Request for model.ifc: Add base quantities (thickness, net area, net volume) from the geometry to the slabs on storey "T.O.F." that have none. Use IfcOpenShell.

First a look at what the model holds.

```python
import ifcopenshell
import ifcopenshell.util.element
import ifcopenshell.util.unit

model = ifcopenshell.open("model.ifc")
print(model.schema)
for unit_type in ("LENGTHUNIT", "AREAUNIT", "VOLUMEUNIT"):
    print(unit_type, ifcopenshell.util.unit.calculate_unit_scale(model, unit_type))
storey = next(s for s in model.by_type("IfcBuildingStorey") if s.Name == "T.O.F.")
slabs = [e for e in ifcopenshell.util.element.get_decomposition(storey) if e.is_a("IfcSlab")]
for e in sorted(slabs, key=lambda e: e.id()):
    print(e.id(), e.is_a(), e.Name, list(ifcopenshell.util.element.get_psets(e, qtos_only=True)), sep=" | ")
```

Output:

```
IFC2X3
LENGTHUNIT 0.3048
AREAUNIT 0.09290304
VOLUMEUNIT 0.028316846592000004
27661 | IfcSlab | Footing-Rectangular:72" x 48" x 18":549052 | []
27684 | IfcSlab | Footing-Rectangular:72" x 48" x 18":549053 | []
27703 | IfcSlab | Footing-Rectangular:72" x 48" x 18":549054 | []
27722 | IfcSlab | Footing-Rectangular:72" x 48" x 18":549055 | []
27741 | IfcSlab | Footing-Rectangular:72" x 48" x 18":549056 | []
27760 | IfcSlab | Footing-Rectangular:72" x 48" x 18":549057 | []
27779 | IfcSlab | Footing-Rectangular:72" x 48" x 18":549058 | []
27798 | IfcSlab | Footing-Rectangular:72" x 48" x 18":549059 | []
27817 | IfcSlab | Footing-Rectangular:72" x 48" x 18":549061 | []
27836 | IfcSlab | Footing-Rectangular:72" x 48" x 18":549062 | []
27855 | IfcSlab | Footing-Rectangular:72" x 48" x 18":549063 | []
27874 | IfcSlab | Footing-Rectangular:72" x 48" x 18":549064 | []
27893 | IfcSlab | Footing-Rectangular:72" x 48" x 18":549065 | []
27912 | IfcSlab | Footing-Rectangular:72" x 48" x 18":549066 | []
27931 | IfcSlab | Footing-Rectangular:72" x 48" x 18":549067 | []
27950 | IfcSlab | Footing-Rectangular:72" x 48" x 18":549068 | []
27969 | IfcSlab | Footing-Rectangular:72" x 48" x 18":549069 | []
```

```python
import ifcopenshell
import ifcopenshell.api.pset
import ifcopenshell.geom
import ifcopenshell.util.element
import ifcopenshell.util.shape
import ifcopenshell.util.unit

model = ifcopenshell.open("model.ifc")
unit_scale = ifcopenshell.util.unit.calculate_unit_scale(model)
area_scale = ifcopenshell.util.unit.calculate_unit_scale(model, "AREAUNIT")
volume_scale = ifcopenshell.util.unit.calculate_unit_scale(model, "VOLUMEUNIT")
settings = ifcopenshell.geom.settings()

storey = next(s for s in model.by_type("IfcBuildingStorey") if s.Name == "T.O.F.")
slabs = [e for e in ifcopenshell.util.element.get_decomposition(storey) if e.is_a("IfcSlab")]

for e in sorted(slabs, key=lambda e: e.id()):
    if ifcopenshell.util.element.get_psets(e, qtos_only=True, should_inherit=False):
        continue
    # Geometry comes back in metres, in the element's own axes.
    shape = ifcopenshell.geom.create_shape(settings, e)
    values = {
        "Width": ifcopenshell.util.shape.get_z(shape.geometry) / unit_scale,
        "NetArea": ifcopenshell.util.shape.get_footprint_area(shape.geometry) / area_scale,
        "NetVolume": ifcopenshell.util.shape.get_volume(shape.geometry) / volume_scale,
    }
    qto = ifcopenshell.api.pset.add_qto(model, product=e, name="BaseQuantities")
    ifcopenshell.api.pset.edit_qto(model, qto=qto, properties=values)
    print(e.id(), {k: round(v, 3) for k, v in values.items()})

model.write("model_rev.ifc")
```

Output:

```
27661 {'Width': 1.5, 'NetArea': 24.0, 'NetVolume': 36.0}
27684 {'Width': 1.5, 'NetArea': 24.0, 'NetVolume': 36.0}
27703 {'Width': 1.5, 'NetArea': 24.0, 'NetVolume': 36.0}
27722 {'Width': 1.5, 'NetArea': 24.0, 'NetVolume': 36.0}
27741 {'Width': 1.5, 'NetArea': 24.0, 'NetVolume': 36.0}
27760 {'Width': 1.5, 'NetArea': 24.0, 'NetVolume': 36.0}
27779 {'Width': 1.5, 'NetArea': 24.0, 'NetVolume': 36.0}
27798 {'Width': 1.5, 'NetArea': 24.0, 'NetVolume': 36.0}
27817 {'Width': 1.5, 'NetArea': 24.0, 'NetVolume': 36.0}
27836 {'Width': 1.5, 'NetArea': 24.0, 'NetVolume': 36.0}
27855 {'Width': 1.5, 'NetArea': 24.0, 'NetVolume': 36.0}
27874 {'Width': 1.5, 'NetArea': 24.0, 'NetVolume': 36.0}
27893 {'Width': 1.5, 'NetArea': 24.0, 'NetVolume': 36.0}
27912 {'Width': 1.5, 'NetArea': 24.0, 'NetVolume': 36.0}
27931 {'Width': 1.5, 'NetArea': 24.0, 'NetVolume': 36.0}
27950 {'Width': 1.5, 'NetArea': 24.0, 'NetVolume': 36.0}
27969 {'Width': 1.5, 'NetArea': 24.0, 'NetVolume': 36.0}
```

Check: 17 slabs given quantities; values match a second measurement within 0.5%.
